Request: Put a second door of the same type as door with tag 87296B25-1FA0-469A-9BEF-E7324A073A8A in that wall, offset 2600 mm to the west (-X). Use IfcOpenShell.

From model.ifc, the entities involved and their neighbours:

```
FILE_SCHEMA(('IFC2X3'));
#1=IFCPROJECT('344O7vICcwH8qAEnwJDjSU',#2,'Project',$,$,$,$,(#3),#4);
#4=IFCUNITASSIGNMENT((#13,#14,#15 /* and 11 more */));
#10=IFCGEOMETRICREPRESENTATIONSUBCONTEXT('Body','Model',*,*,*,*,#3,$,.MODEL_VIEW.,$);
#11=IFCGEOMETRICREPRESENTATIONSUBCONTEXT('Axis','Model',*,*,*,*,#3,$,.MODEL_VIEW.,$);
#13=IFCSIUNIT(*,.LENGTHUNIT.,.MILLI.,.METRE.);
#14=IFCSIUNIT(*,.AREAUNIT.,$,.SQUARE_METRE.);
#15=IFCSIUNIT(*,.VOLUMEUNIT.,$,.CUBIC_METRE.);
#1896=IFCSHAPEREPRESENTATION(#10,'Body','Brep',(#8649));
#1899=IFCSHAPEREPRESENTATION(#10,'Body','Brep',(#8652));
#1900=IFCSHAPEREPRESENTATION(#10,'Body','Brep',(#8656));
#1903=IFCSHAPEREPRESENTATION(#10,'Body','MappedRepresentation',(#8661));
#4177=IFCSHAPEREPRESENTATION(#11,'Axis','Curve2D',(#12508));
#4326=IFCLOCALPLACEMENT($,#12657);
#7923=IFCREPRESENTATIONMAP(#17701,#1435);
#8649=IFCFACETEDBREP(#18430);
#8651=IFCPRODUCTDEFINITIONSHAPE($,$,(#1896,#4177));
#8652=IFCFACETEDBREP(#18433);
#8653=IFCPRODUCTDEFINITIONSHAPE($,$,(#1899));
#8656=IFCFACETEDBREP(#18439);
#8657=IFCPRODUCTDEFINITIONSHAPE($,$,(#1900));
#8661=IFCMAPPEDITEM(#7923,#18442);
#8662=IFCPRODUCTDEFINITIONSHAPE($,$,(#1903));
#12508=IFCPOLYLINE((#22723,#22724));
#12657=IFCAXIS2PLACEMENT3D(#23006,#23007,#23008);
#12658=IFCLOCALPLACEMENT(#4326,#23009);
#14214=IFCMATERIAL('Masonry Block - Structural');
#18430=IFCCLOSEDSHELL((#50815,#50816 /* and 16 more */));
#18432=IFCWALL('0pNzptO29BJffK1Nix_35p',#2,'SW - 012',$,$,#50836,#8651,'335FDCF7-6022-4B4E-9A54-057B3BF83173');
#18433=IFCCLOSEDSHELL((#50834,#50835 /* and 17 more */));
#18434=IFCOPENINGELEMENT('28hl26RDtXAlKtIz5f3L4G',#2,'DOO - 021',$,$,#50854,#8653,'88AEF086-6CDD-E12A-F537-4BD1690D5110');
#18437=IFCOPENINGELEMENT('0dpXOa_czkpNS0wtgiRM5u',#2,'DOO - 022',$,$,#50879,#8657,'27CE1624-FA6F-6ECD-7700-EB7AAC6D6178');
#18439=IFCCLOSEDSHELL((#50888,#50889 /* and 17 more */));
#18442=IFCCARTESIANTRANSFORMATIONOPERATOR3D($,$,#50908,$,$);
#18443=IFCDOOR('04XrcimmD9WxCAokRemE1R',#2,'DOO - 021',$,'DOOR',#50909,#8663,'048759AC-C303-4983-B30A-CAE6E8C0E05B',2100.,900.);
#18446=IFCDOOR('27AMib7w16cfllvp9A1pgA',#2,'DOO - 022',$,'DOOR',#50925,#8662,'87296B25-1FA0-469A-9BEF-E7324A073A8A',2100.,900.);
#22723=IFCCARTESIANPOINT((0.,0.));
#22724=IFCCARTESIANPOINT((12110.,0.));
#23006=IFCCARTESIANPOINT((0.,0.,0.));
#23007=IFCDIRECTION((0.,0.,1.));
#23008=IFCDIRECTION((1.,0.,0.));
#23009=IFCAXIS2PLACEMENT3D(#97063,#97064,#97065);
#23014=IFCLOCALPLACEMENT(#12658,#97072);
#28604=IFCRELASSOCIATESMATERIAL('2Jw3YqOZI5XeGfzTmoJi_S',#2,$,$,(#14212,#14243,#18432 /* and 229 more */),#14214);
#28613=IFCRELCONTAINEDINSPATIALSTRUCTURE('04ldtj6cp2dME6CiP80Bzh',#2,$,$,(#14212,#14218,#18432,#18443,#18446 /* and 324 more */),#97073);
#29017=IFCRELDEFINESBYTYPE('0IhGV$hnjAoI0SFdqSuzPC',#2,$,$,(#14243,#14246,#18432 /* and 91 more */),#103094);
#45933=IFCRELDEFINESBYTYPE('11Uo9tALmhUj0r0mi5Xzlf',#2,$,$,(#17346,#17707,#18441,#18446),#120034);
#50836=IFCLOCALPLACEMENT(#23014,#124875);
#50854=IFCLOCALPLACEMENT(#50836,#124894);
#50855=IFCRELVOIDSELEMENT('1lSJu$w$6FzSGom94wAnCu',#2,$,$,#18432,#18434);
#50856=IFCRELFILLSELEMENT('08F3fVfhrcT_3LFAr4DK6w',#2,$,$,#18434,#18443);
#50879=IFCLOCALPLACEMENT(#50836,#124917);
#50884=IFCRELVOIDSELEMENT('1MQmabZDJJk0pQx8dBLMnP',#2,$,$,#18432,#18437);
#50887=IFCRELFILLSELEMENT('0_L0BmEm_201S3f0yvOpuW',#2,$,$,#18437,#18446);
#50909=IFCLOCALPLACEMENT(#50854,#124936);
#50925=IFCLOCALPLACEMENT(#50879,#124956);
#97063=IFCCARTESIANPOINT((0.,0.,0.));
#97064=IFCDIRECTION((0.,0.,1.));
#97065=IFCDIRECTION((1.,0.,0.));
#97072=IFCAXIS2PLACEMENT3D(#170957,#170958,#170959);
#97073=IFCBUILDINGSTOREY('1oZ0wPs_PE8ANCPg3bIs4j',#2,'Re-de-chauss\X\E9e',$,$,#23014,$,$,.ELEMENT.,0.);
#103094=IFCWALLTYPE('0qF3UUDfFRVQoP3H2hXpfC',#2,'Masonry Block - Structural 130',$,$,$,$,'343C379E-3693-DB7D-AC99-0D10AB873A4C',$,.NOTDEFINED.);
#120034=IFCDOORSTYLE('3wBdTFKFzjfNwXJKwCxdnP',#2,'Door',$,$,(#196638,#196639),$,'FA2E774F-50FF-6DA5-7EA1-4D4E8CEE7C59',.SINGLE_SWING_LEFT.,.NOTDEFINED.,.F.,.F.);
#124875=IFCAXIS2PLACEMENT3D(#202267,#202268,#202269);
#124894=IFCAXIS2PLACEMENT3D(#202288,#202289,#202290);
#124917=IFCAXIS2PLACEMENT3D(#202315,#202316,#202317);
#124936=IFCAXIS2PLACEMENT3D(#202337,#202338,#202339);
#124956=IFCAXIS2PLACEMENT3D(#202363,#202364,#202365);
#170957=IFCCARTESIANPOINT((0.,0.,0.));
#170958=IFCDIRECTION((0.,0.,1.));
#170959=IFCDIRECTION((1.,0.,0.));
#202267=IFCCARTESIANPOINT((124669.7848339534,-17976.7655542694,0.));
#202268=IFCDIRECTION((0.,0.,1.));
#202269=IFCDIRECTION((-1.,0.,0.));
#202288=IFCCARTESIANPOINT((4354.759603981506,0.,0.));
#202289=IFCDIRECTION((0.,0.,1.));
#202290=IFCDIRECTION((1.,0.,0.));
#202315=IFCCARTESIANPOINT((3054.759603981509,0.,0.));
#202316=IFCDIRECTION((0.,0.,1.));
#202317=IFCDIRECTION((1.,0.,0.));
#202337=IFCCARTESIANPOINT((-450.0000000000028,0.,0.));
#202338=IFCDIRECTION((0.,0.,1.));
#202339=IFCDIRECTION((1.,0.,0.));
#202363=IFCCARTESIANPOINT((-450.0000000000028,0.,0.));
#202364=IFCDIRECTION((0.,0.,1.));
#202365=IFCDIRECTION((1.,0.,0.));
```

```python
import ifcopenshell
import ifcopenshell.api.feature
import ifcopenshell.api.geometry
import ifcopenshell.api.root
import ifcopenshell.geom
import ifcopenshell.util.element
import ifcopenshell.util.placement
import ifcopenshell.util.shape
import ifcopenshell.util.unit

model = ifcopenshell.open("model.ifc")
unit_scale = ifcopenshell.util.unit.calculate_unit_scale(model)
settings = ifcopenshell.geom.settings()


def volume(element):
    """Net volume in cubic metres, openings subtracted."""
    shape = ifcopenshell.geom.create_shape(settings, element)
    return ifcopenshell.util.shape.get_volume(shape.geometry)


def reuse_history(source, copy):
    """copy_class also copies each property set's owner history, people and application; keep the originals."""
    for rel in copy.IsDefinedBy:
        if rel.is_a("IfcRelDefinesByProperties") and (history := rel.RelatingPropertyDefinition.OwnerHistory):
            rel.RelatingPropertyDefinition.OwnerHistory = source.OwnerHistory
            ifcopenshell.util.element.remove_deep2(model, history)


door = model.by_guid("27AMib7w16cfllvp9A1pgA")
opening = door.FillsVoids[0].RelatingOpeningElement
wall = opening.VoidsElements[0].RelatingBuildingElement
before = volume(wall)
shift = ifcopenshell.util.placement.get_local_placement(wall.ObjectPlacement)[:3, 0] * 2.6 / unit_scale

# copy_class copies the void relationship, type, container and properties, but no geometry.
new_opening = ifcopenshell.api.root.copy_class(model, product=opening)
new_opening.Representation = ifcopenshell.util.element.copy_deep(
    model, opening.Representation, exclude=["IfcGeometricRepresentationContext", "IfcRepresentationMap"]
)
new_opening.Tag = None
new_door = ifcopenshell.api.root.copy_class(model, product=door)
new_door.Representation = ifcopenshell.util.element.copy_deep(
    model, door.Representation, exclude=["IfcGeometricRepresentationContext", "IfcRepresentationMap"]
)
new_door.Tag = None
reuse_history(door, new_door)
fills = ifcopenshell.api.feature.add_filling(model, opening=new_opening, element=new_door)
fills.OwnerHistory = new_door.OwnerHistory  # required in IFC2X3

for old, new in ((opening, new_opening), (door, new_door)):
    matrix = ifcopenshell.util.placement.get_local_placement(old.ObjectPlacement)
    matrix[:3, 3] += shift
    ifcopenshell.api.geometry.edit_object_placement(model, product=new, matrix=matrix, is_si=False)

after = volume(wall)

print(f"wall volume {before:.3f} -> {after:.3f} m3")

model.write("model_v2.ifc")
```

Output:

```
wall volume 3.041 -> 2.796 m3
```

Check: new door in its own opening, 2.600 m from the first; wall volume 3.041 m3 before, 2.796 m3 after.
